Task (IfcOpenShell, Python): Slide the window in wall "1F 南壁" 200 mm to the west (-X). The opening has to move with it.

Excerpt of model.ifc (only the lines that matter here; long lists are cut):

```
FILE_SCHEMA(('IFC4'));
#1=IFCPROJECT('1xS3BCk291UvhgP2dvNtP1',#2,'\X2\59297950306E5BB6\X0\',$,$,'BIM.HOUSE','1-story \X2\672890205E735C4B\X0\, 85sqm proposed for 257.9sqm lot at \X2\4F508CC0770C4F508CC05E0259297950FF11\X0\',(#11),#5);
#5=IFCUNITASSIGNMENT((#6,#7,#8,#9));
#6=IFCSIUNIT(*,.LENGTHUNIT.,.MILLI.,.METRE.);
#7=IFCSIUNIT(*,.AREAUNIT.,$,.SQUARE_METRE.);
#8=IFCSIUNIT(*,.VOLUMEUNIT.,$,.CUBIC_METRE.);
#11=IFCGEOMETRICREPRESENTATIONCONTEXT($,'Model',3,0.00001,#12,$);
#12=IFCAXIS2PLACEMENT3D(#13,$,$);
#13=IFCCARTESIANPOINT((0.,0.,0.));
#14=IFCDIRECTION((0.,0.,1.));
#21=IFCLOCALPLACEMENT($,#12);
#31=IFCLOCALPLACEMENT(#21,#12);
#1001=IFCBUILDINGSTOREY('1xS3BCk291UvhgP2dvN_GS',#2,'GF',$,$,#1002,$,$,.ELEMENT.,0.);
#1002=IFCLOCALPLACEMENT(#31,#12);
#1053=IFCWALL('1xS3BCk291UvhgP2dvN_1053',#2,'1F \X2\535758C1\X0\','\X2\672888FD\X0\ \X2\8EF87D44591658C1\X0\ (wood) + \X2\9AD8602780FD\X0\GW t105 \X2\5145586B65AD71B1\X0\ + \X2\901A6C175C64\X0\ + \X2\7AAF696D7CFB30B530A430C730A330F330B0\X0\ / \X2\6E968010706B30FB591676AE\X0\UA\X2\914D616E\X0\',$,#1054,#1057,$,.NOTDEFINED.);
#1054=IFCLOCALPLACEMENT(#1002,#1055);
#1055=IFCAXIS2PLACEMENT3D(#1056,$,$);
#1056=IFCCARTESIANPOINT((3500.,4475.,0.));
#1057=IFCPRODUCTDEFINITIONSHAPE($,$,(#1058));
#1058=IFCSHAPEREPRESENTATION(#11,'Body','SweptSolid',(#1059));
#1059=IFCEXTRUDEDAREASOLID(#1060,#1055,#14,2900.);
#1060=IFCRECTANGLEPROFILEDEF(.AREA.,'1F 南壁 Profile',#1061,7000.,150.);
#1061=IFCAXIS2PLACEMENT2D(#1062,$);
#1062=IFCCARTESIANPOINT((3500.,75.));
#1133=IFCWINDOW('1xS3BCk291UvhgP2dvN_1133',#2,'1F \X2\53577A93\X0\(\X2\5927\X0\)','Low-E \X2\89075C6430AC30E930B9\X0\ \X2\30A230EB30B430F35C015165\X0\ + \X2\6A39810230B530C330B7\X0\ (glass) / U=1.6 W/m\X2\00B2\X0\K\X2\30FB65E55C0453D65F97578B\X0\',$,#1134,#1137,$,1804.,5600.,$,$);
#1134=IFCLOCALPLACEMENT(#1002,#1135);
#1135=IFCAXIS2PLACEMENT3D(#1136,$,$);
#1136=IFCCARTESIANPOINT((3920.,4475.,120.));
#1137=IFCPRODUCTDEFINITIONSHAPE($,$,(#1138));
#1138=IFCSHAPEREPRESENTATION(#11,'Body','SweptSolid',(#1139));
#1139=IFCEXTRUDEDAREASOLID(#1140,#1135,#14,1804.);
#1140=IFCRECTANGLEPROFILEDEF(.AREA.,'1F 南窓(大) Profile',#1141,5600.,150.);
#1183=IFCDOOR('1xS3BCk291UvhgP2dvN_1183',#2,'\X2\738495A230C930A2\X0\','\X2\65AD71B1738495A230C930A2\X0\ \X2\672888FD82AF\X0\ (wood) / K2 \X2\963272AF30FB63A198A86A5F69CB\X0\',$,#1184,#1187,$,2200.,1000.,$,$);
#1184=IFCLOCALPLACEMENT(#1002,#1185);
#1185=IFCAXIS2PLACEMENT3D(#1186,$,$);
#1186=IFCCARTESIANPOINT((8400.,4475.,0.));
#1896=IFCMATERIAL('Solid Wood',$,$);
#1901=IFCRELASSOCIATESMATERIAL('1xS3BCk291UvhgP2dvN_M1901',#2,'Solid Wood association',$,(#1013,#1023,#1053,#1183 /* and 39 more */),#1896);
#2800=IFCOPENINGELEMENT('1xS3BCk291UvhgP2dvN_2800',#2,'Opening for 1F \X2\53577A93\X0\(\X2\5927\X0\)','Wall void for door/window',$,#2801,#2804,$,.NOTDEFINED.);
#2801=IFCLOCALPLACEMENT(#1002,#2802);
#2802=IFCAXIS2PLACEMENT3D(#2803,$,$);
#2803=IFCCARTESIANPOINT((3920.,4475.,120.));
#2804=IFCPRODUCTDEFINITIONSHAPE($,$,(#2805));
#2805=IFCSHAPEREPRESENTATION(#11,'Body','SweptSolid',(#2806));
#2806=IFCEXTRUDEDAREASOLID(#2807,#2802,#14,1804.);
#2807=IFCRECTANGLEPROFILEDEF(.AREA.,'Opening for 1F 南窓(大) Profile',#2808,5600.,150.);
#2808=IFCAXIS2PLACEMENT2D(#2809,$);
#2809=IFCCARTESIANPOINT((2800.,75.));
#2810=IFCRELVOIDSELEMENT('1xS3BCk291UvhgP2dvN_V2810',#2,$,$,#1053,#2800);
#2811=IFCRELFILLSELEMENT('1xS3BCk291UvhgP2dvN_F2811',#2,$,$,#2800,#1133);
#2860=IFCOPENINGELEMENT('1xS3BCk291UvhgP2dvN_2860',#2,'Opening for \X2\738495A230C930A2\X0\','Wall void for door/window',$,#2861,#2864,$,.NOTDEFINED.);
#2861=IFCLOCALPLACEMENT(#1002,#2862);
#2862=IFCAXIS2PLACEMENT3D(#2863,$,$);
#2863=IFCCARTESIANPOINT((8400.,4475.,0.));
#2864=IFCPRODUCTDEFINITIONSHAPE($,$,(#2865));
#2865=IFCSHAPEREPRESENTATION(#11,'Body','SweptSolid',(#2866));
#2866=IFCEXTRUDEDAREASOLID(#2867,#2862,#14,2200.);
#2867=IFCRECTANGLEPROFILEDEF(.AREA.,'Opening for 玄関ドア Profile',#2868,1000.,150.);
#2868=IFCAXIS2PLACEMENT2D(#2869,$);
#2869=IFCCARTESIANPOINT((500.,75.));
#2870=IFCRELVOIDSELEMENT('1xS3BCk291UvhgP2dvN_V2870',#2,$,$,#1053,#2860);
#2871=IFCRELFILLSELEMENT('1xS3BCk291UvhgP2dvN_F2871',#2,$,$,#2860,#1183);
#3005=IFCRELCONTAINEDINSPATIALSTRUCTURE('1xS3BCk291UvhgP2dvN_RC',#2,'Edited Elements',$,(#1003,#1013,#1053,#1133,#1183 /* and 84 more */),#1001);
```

```python
import ifcopenshell
import ifcopenshell.api.geometry
import ifcopenshell.util.placement
import ifcopenshell.util.unit

model = ifcopenshell.open("model.ifc")
unit_scale = ifcopenshell.util.unit.calculate_unit_scale(model)

window = model.by_guid("1xS3BCk291UvhgP2dvN_1133")
opening = window.FillsVoids[0].RelatingOpeningElement
wall = opening.VoidsElements[0].RelatingBuildingElement

wall_matrix = ifcopenshell.util.placement.get_local_placement(wall.ObjectPlacement)
shift = wall_matrix[:3, 0] * -0.2 / unit_scale
before = ifcopenshell.util.placement.get_local_placement(window.ObjectPlacement)[:3, 3].copy()

# The window is not placed relative to its opening, so move both.
for product in (opening, window):
    matrix = ifcopenshell.util.placement.get_local_placement(product.ObjectPlacement)
    matrix[:3, 3] += shift
    ifcopenshell.api.geometry.edit_object_placement(model, product=product, matrix=matrix, is_si=False)

after = ifcopenshell.util.placement.get_local_placement(window.ObjectPlacement)[:3, 3]
print("window moved by", (after - before).round(3) + 0.0)

model.write("model_v2.ifc")
```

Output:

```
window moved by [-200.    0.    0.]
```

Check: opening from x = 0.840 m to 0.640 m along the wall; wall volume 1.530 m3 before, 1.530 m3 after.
